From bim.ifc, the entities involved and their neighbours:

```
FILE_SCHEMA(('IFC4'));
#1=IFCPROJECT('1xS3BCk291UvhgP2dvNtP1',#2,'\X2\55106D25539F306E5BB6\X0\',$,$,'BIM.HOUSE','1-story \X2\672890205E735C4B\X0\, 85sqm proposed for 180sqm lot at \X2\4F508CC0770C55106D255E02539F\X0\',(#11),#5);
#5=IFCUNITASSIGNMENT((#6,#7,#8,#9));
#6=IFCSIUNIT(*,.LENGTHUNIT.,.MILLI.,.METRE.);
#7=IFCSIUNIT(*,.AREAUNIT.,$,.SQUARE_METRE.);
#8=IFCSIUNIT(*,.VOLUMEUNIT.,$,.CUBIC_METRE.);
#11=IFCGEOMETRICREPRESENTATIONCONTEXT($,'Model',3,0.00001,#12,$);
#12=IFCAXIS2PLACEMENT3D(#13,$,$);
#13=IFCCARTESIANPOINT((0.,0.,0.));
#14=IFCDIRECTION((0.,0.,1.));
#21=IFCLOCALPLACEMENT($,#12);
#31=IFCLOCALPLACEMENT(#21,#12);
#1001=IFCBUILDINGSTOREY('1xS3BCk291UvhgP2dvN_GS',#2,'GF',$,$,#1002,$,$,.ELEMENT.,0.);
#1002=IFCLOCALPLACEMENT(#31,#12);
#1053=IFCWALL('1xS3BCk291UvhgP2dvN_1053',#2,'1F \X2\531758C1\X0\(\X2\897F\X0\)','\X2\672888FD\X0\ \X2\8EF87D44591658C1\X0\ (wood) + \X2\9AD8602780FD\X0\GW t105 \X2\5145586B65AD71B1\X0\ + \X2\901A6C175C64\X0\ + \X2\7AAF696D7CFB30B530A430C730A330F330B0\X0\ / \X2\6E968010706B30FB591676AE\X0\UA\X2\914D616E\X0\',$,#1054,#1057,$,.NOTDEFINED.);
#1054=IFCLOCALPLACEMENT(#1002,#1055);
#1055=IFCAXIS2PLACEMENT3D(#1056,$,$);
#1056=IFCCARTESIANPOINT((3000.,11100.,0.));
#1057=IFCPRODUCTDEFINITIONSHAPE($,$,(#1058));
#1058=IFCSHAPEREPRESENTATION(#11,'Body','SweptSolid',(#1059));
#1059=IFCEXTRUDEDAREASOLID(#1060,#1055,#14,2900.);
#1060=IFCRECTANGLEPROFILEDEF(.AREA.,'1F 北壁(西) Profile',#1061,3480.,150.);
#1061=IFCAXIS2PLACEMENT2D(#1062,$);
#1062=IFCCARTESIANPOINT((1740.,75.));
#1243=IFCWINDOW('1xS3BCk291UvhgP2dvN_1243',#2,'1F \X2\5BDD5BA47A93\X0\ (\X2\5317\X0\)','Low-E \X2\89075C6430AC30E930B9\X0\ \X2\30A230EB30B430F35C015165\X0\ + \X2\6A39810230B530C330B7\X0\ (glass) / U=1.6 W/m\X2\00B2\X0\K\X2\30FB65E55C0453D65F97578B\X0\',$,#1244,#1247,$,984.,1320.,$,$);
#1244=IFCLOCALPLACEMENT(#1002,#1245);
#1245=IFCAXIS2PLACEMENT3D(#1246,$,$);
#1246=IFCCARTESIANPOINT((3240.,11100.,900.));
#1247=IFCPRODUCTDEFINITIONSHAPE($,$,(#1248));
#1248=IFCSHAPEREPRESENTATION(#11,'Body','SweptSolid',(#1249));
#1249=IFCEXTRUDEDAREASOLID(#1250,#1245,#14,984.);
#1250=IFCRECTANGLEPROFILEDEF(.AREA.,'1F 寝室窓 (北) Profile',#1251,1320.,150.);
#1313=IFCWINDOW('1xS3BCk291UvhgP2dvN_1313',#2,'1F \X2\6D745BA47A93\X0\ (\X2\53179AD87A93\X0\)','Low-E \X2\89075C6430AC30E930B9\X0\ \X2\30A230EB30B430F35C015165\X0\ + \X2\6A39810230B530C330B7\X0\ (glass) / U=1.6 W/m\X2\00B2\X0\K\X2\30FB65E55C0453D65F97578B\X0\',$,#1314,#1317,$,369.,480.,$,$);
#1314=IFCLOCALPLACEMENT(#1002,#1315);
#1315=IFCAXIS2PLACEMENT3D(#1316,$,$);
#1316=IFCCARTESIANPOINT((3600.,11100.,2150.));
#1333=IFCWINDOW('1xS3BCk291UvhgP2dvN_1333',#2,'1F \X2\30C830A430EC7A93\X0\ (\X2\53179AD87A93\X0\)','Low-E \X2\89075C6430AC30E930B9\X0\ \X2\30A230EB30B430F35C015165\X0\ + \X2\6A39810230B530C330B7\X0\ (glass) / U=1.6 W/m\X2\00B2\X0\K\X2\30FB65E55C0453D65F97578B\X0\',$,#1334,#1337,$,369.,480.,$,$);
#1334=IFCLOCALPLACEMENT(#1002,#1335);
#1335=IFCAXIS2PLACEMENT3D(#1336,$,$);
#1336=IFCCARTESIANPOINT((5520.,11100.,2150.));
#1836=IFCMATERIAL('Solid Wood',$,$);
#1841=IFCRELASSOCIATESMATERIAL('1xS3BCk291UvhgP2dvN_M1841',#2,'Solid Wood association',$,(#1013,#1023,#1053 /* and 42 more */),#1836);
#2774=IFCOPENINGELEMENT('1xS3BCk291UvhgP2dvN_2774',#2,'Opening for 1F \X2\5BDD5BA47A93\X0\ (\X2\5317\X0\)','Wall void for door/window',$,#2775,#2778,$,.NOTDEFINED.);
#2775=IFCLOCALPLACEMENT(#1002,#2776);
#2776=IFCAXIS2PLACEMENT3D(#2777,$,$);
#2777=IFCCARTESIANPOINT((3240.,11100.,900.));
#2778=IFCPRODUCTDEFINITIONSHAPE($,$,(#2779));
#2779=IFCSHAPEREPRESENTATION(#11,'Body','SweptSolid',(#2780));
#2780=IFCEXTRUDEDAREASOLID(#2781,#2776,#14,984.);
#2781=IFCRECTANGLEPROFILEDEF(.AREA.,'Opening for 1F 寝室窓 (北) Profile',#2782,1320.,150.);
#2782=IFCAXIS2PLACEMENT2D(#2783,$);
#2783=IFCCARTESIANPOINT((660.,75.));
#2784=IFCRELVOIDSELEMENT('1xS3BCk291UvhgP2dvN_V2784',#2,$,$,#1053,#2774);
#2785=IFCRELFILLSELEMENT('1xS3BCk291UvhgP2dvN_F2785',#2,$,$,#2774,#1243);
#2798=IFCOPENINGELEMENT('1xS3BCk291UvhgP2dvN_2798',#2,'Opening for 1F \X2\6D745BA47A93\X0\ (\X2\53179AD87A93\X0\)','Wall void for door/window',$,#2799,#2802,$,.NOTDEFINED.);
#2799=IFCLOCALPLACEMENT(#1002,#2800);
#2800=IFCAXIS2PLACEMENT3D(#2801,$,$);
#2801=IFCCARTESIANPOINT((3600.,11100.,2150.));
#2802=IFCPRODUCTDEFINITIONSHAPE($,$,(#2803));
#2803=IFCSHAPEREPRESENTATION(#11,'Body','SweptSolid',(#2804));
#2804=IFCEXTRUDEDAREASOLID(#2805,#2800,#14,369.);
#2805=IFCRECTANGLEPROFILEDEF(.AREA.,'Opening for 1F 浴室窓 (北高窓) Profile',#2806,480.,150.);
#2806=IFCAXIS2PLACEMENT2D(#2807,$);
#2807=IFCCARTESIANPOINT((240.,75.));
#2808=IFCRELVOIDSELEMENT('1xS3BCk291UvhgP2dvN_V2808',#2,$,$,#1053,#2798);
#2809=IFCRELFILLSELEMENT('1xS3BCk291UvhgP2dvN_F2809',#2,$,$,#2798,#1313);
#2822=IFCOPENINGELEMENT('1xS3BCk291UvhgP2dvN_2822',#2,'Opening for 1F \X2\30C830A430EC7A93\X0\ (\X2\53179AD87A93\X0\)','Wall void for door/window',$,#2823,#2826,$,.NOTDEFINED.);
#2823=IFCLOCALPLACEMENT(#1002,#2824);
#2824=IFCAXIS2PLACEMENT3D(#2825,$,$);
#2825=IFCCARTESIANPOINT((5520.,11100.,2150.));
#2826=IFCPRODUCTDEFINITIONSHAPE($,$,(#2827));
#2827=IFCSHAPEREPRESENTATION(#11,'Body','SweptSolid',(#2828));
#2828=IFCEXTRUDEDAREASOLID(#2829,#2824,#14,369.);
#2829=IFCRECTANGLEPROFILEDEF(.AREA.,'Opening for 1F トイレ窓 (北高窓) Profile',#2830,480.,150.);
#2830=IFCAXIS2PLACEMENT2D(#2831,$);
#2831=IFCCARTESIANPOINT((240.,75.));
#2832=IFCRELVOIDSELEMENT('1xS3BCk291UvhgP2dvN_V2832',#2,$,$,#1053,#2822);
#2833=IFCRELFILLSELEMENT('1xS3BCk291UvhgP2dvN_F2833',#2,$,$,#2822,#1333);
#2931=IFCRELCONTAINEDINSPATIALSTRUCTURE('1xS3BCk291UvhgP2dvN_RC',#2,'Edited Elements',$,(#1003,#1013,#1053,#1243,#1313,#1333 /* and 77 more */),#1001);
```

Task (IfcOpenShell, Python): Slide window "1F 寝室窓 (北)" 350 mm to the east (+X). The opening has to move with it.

```python
import ifcopenshell
import ifcopenshell.api.geometry
import ifcopenshell.util.placement
import ifcopenshell.util.unit

model = ifcopenshell.open("bim.ifc")
unit_scale = ifcopenshell.util.unit.calculate_unit_scale(model)

window = model.by_guid("1xS3BCk291UvhgP2dvN_1243")
opening = window.FillsVoids[0].RelatingOpeningElement
wall = opening.VoidsElements[0].RelatingBuildingElement

wall_matrix = ifcopenshell.util.placement.get_local_placement(wall.ObjectPlacement)
shift = wall_matrix[:3, 0] * 0.35 / unit_scale
before = ifcopenshell.util.placement.get_local_placement(window.ObjectPlacement)[:3, 3].copy()

# The window is not placed relative to its opening, so move both.
for product in (opening, window):
    matrix = ifcopenshell.util.placement.get_local_placement(product.ObjectPlacement)
    matrix[:3, 3] += shift
    ifcopenshell.api.geometry.edit_object_placement(model, product=product, matrix=matrix, is_si=False)

after = ifcopenshell.util.placement.get_local_placement(window.ObjectPlacement)[:3, 3]
print("window moved by", (after - before).round(3) + 0.0)

model.write("bim-out.ifc")
```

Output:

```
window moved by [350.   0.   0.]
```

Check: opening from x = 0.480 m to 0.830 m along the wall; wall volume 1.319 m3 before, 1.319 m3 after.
